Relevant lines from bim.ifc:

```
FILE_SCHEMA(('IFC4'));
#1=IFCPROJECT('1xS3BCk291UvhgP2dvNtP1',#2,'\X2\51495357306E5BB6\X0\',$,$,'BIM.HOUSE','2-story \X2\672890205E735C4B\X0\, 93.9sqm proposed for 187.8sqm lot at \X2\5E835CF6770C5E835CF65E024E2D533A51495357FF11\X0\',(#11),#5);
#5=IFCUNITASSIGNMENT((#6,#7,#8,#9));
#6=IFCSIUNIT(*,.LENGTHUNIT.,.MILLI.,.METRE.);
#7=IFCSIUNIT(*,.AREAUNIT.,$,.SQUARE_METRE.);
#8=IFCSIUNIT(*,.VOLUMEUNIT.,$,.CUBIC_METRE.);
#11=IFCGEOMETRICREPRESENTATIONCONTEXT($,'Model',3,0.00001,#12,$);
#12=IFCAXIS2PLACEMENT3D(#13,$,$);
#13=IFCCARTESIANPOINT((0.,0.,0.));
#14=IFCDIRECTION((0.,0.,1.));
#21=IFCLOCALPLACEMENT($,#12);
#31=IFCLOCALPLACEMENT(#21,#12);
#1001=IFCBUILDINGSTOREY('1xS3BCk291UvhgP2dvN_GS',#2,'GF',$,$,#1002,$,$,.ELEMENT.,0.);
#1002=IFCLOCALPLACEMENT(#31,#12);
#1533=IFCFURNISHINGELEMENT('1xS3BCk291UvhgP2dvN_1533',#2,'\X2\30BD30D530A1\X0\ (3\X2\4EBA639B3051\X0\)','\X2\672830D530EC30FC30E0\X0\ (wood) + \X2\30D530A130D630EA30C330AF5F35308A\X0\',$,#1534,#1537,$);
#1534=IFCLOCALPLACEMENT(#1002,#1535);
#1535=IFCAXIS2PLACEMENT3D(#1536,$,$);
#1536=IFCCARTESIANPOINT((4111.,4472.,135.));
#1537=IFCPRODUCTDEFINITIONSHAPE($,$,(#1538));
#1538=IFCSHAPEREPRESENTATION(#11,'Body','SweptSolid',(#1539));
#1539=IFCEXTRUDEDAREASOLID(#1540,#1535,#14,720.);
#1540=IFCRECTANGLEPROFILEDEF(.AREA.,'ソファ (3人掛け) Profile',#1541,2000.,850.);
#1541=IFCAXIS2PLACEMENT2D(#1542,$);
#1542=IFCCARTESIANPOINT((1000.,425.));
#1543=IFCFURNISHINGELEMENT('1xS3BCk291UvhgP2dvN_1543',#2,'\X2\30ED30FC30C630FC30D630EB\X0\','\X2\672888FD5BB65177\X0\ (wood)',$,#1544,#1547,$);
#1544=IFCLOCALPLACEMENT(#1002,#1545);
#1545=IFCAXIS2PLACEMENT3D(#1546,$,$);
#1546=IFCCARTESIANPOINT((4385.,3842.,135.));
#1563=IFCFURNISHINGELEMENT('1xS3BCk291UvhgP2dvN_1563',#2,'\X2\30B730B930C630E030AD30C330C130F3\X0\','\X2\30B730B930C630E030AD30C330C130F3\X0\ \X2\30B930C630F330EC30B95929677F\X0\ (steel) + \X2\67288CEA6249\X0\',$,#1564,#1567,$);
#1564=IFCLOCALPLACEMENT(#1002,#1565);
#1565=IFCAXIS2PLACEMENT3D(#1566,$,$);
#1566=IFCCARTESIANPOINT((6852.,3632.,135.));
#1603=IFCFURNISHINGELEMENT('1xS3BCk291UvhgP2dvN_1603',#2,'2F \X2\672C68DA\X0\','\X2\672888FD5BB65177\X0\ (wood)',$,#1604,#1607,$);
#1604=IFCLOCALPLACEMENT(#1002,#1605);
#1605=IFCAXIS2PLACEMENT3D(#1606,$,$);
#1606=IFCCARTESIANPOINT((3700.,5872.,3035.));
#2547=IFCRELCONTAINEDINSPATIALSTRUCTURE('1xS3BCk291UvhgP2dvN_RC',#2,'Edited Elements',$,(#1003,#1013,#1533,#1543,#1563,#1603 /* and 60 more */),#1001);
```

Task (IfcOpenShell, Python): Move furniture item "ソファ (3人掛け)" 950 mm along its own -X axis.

```python
import ifcopenshell
import ifcopenshell.api.geometry
import ifcopenshell.util.placement

model = ifcopenshell.open("bim.ifc")

item = model.by_guid("1xS3BCk291UvhgP2dvN_1533")
matrix = ifcopenshell.util.placement.get_local_placement(item.ObjectPlacement)
matrix[:3, 3] -= matrix[:3, 0] * 950.0
ifcopenshell.api.geometry.edit_object_placement(model, product=item, matrix=matrix, is_si=False)

print(ifcopenshell.util.placement.get_local_placement(item.ObjectPlacement).round(3) + 0.0)

model.write("bim_rev.ifc")
```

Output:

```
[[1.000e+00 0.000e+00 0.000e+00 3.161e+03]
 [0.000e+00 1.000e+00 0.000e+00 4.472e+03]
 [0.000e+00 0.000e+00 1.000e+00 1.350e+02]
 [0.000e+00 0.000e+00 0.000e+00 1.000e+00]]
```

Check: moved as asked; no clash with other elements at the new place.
